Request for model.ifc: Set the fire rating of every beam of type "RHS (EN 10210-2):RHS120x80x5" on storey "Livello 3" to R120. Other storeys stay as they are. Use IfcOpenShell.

First a look at what the model holds.

```python
import ifcopenshell
import ifcopenshell.util.element

model = ifcopenshell.open("model.ifc")
print(model.schema)
storey = next(s for s in model.by_type("IfcBuildingStorey") if s.Name == "Livello 3")
beams = [e for e in ifcopenshell.util.element.get_decomposition(storey) if e.is_a("IfcBeam")]
seen = {}
for e in beams:
    element_type = ifcopenshell.util.element.get_type(e)
    key = (element_type.Name if element_type != e and element_type else None, ifcopenshell.util.element.get_pset(e, "Pset_BeamCommon", "FireRating"))
    seen[key] = seen.get(key, 0) + 1
for (name, value), count in sorted(seen.items(), key=str):
    print(count, "x", name, "|", value)
```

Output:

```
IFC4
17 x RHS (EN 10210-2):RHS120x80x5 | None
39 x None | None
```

```python
import ifcopenshell
import ifcopenshell.api.pset
import ifcopenshell.util.element

model = ifcopenshell.open("model.ifc")

storey = next(s for s in model.by_type("IfcBuildingStorey") if s.Name == "Livello 3")
beams = [e for e in ifcopenshell.util.element.get_decomposition(storey) if e.is_a("IfcBeam")]

count = 0
for e in beams:
    element_type = ifcopenshell.util.element.get_type(e)
    if element_type in (None, e) or element_type.Name != "RHS (EN 10210-2):RHS120x80x5":
        continue
    # add_pset returns the element's existing set when there is one.
    pset = ifcopenshell.api.pset.add_pset(model, product=e, name="Pset_BeamCommon")
    ifcopenshell.api.pset.edit_pset(model, pset=pset, properties={"FireRating": "R120"})
    count += 1

print(count, "beams updated")

model.write("model_edited.ifc")
```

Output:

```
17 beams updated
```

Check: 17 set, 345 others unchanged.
